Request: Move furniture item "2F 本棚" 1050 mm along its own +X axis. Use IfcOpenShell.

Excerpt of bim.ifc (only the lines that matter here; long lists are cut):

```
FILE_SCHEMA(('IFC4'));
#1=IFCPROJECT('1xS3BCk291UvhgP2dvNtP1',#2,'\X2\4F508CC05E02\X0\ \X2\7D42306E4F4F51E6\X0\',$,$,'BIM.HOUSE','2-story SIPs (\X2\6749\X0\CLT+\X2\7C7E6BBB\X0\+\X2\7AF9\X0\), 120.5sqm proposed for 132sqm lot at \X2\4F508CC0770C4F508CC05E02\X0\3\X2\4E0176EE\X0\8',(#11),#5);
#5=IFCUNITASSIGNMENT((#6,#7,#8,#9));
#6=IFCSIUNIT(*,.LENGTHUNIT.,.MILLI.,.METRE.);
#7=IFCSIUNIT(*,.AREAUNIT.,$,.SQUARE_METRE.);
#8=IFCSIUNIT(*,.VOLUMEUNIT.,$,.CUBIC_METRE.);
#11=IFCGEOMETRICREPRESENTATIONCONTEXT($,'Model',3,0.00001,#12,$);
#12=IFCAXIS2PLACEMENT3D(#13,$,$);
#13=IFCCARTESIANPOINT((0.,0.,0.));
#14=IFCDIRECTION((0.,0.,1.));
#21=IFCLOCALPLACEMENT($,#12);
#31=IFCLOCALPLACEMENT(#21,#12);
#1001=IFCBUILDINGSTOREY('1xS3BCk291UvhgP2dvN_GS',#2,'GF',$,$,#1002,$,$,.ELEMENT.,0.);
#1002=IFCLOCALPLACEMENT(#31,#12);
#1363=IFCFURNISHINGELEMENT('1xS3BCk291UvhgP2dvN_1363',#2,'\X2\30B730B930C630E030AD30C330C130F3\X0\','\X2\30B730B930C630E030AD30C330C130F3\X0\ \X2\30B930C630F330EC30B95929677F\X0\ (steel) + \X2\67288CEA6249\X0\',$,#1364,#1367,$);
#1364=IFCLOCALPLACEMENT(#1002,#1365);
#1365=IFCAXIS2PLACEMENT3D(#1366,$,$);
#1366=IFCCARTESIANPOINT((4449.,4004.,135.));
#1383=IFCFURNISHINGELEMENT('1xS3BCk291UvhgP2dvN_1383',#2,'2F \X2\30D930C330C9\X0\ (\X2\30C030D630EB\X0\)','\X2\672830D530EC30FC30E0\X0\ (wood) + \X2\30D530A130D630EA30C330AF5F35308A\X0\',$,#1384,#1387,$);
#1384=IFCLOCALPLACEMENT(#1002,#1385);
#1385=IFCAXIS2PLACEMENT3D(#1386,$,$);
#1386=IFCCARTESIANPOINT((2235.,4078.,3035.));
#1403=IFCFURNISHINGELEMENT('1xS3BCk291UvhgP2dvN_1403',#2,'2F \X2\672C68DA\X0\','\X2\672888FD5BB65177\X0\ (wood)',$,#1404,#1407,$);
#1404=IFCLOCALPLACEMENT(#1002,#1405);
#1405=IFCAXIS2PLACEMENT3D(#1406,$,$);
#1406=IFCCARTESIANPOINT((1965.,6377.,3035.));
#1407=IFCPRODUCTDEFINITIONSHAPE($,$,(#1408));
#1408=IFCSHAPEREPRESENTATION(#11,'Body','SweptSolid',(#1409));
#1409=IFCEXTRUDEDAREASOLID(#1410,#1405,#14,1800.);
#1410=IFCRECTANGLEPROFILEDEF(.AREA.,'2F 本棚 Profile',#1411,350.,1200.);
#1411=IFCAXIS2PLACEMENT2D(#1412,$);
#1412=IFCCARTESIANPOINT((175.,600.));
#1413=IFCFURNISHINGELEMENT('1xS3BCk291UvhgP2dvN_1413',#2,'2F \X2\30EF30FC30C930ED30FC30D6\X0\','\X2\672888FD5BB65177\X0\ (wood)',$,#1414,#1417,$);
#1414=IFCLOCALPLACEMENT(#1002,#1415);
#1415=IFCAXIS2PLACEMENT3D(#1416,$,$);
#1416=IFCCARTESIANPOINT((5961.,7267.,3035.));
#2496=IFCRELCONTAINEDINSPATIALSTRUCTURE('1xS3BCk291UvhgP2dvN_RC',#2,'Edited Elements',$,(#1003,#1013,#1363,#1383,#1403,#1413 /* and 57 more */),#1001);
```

```python
import ifcopenshell
import ifcopenshell.api.geometry
import ifcopenshell.util.placement
import ifcopenshell.util.unit

model = ifcopenshell.open("bim.ifc")
unit_scale = ifcopenshell.util.unit.calculate_unit_scale(model)

item = model.by_guid("1xS3BCk291UvhgP2dvN_1403")
matrix = ifcopenshell.util.placement.get_local_placement(item.ObjectPlacement)
matrix[:3, 3] += matrix[:3, 0] * 1.05 / unit_scale
ifcopenshell.api.geometry.edit_object_placement(model, product=item, matrix=matrix, is_si=False)

print(ifcopenshell.util.placement.get_local_placement(item.ObjectPlacement).round(3) + 0.0)

model.write("bim_edited.ifc")
```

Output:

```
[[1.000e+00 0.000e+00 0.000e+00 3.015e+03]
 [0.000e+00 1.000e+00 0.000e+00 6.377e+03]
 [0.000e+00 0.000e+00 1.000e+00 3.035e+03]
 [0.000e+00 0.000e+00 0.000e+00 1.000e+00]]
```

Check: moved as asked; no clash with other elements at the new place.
